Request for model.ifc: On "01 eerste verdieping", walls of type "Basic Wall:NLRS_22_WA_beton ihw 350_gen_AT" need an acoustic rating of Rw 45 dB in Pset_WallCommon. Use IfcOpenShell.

First a look at what the model holds.

```python
import ifcopenshell
import ifcopenshell.util.element

model = ifcopenshell.open("model.ifc")
print(model.schema)
storey = next(s for s in model.by_type("IfcBuildingStorey") if s.Name == "01 eerste verdieping")
walls = [e for e in ifcopenshell.util.element.get_decomposition(storey) if e.is_a("IfcWall")]
seen = {}
for e in walls:
    element_type = ifcopenshell.util.element.get_type(e)
    key = (element_type.Name if element_type != e and element_type else None, ifcopenshell.util.element.get_pset(e, "Pset_WallCommon", "AcousticRating"))
    seen[key] = seen.get(key, 0) + 1
for (name, value), count in sorted(seen.items(), key=str):
    print(count, "x", name, "|", value)
```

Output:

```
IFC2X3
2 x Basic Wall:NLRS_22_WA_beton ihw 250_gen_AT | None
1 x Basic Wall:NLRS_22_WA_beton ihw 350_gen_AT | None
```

```python
import ifcopenshell
import ifcopenshell.api.pset
import ifcopenshell.util.element

model = ifcopenshell.open("model.ifc")

storey = next(s for s in model.by_type("IfcBuildingStorey") if s.Name == "01 eerste verdieping")
walls = [e for e in ifcopenshell.util.element.get_decomposition(storey) if e.is_a("IfcWall")]

count = 0
for e in walls:
    element_type = ifcopenshell.util.element.get_type(e)
    if element_type in (None, e) or element_type.Name != "Basic Wall:NLRS_22_WA_beton ihw 350_gen_AT":
        continue
    found = ifcopenshell.util.element.get_pset(e, "Pset_WallCommon", should_inherit=False)
    if found:
        pset = model.by_id(found["id"])
        if len(ifcopenshell.util.element.get_elements_by_pset(pset)) > 1:
            pset = ifcopenshell.api.pset.unshare_pset(model, products=[e], pset=pset)[0]
    else:
        pset = ifcopenshell.api.pset.add_pset(model, product=e, name="Pset_WallCommon")
    ifcopenshell.api.pset.edit_pset(model, pset=pset, properties={"AcousticRating": "Rw 45 dB"})
    count += 1

print(count, "walls updated")

model.write("model-out.ifc")
```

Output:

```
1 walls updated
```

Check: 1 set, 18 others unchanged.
